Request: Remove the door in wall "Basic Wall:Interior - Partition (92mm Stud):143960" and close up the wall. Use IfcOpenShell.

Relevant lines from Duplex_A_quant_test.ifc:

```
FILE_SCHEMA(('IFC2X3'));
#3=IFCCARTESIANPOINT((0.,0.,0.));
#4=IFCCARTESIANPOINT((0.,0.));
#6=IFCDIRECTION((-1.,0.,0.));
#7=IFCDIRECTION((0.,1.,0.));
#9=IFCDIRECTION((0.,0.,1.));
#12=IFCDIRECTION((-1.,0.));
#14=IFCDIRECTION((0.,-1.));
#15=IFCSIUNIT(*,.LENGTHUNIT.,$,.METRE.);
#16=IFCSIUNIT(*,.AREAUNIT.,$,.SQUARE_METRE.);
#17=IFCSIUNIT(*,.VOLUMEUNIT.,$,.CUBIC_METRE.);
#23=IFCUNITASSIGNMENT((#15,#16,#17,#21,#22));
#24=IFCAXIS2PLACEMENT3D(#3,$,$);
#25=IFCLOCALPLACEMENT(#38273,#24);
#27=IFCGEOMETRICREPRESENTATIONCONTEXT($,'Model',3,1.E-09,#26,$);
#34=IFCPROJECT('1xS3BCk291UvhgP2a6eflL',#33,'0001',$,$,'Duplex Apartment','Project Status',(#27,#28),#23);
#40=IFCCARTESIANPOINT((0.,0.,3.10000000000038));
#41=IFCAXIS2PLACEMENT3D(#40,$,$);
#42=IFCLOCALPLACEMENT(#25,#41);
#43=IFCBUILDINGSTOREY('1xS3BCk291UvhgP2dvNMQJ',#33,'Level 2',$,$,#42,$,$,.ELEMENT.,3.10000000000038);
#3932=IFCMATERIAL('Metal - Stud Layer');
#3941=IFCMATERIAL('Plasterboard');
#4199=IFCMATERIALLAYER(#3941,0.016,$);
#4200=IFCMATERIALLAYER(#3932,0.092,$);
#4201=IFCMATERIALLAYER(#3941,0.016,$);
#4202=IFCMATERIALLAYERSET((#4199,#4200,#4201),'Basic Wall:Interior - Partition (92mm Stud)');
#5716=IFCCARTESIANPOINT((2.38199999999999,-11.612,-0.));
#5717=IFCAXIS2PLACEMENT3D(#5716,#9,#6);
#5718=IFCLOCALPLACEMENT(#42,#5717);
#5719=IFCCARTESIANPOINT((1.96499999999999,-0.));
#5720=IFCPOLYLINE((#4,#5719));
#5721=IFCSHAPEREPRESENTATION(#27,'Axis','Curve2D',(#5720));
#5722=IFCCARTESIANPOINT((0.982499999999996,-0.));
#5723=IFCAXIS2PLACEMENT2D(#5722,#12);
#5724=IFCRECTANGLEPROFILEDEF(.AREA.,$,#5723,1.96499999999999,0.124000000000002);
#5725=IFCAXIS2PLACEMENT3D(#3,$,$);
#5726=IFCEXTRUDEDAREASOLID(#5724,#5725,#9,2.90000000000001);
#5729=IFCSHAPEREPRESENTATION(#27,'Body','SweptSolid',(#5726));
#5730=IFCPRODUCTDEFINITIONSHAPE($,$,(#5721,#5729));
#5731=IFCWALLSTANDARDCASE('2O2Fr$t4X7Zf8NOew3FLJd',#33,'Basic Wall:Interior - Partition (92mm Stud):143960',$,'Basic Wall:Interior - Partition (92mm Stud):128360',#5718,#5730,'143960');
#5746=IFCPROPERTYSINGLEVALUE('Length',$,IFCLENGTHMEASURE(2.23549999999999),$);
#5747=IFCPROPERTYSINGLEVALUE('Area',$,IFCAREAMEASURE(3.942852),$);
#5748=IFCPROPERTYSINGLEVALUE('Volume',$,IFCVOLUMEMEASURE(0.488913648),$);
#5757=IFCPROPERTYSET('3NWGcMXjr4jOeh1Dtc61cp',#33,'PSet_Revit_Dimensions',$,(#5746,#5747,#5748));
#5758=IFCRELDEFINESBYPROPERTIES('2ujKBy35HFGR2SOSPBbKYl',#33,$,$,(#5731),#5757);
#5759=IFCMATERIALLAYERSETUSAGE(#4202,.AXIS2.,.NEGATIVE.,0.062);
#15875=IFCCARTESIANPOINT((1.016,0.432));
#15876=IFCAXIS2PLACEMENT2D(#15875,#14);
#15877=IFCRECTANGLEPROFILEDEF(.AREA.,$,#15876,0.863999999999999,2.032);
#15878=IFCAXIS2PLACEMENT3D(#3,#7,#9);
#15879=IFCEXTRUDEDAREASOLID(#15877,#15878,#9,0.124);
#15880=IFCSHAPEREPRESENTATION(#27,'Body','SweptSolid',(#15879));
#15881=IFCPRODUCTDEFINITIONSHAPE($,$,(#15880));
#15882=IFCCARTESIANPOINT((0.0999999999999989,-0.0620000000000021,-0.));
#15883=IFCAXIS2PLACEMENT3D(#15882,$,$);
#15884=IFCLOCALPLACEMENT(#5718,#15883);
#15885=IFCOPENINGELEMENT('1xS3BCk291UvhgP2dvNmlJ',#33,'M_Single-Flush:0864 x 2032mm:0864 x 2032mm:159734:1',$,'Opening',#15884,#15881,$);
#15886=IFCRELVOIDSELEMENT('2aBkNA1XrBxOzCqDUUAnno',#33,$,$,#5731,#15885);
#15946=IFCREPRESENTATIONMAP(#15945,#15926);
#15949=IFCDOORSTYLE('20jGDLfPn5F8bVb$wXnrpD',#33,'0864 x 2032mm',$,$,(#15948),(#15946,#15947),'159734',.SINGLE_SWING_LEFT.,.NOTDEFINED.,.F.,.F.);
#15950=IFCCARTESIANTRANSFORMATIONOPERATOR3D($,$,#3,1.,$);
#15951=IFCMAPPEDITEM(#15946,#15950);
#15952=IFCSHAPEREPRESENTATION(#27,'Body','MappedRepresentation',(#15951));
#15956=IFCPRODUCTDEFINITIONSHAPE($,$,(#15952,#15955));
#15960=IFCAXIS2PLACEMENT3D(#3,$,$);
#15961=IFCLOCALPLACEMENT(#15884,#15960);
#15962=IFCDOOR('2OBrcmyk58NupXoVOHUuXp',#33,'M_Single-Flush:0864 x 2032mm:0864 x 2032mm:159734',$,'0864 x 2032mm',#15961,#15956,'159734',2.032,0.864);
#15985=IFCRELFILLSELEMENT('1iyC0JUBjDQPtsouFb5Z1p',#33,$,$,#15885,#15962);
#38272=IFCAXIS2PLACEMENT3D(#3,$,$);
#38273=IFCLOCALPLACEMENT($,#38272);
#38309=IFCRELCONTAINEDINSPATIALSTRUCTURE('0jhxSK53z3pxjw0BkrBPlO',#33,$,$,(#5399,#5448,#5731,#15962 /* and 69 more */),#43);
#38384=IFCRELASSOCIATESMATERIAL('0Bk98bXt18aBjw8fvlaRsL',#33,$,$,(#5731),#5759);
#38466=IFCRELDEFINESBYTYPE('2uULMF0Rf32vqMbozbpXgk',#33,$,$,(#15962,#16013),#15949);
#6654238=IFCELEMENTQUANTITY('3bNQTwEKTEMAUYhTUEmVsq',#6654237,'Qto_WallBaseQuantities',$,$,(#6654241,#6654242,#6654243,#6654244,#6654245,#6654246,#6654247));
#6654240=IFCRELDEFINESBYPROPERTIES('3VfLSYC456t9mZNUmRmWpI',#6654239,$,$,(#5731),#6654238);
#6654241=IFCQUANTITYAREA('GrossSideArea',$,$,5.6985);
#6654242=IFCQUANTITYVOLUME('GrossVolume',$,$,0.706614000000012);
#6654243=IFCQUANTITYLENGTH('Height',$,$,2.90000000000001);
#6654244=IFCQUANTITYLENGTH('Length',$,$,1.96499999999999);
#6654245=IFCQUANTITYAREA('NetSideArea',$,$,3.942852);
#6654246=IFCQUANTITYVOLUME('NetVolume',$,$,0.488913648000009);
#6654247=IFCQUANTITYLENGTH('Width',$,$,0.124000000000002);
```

```python
import ifcopenshell
import ifcopenshell.api.feature
import ifcopenshell.api.pset
import ifcopenshell.api.root
import ifcopenshell.geom
import ifcopenshell.util.element
import ifcopenshell.util.shape
import ifcopenshell.util.unit

model = ifcopenshell.open("Duplex_A_quant_test.ifc")
area_scale = ifcopenshell.util.unit.calculate_unit_scale(model, "AREAUNIT")
volume_scale = ifcopenshell.util.unit.calculate_unit_scale(model, "VOLUMEUNIT")
settings = ifcopenshell.geom.settings()


def volume(element):
    """Net volume in cubic metres, openings subtracted."""
    shape = ifcopenshell.geom.create_shape(settings, element)
    return ifcopenshell.util.shape.get_volume(shape.geometry)


door = model.by_guid("2OBrcmyk58NupXoVOHUuXp")
opening = door.FillsVoids[0].RelatingOpeningElement
wall = opening.VoidsElements[0].RelatingBuildingElement
before = volume(wall)

ifcopenshell.api.root.remove_product(model, product=door)
ifcopenshell.api.feature.remove_feature(model, feature=opening)

after = volume(wall)
thickness = 0.124  # wall thickness in metres

# Update the wall's stored quantities.
pset = model.by_id(ifcopenshell.util.element.get_pset(wall, "PSet_Revit_Dimensions", should_inherit=False)["id"])
ifcopenshell.api.pset.edit_pset(model, pset=pset, properties={
    "Area": model.create_entity("IfcAreaMeasure", after / thickness / area_scale),
    "Volume": model.create_entity("IfcVolumeMeasure", after / volume_scale),
})
qto = model.by_id(ifcopenshell.util.element.get_pset(wall, "Qto_WallBaseQuantities", should_inherit=False)["id"])
ifcopenshell.api.pset.edit_qto(model, qto=qto, properties={
    "NetSideArea": after / thickness / area_scale,
    "NetVolume": after / volume_scale,
})

print(f"wall volume {before:.3f} -> {after:.3f} m3")

model.write("Duplex_A_quant_test_v2.ifc")
```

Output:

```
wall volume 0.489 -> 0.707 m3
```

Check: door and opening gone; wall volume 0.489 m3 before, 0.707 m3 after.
